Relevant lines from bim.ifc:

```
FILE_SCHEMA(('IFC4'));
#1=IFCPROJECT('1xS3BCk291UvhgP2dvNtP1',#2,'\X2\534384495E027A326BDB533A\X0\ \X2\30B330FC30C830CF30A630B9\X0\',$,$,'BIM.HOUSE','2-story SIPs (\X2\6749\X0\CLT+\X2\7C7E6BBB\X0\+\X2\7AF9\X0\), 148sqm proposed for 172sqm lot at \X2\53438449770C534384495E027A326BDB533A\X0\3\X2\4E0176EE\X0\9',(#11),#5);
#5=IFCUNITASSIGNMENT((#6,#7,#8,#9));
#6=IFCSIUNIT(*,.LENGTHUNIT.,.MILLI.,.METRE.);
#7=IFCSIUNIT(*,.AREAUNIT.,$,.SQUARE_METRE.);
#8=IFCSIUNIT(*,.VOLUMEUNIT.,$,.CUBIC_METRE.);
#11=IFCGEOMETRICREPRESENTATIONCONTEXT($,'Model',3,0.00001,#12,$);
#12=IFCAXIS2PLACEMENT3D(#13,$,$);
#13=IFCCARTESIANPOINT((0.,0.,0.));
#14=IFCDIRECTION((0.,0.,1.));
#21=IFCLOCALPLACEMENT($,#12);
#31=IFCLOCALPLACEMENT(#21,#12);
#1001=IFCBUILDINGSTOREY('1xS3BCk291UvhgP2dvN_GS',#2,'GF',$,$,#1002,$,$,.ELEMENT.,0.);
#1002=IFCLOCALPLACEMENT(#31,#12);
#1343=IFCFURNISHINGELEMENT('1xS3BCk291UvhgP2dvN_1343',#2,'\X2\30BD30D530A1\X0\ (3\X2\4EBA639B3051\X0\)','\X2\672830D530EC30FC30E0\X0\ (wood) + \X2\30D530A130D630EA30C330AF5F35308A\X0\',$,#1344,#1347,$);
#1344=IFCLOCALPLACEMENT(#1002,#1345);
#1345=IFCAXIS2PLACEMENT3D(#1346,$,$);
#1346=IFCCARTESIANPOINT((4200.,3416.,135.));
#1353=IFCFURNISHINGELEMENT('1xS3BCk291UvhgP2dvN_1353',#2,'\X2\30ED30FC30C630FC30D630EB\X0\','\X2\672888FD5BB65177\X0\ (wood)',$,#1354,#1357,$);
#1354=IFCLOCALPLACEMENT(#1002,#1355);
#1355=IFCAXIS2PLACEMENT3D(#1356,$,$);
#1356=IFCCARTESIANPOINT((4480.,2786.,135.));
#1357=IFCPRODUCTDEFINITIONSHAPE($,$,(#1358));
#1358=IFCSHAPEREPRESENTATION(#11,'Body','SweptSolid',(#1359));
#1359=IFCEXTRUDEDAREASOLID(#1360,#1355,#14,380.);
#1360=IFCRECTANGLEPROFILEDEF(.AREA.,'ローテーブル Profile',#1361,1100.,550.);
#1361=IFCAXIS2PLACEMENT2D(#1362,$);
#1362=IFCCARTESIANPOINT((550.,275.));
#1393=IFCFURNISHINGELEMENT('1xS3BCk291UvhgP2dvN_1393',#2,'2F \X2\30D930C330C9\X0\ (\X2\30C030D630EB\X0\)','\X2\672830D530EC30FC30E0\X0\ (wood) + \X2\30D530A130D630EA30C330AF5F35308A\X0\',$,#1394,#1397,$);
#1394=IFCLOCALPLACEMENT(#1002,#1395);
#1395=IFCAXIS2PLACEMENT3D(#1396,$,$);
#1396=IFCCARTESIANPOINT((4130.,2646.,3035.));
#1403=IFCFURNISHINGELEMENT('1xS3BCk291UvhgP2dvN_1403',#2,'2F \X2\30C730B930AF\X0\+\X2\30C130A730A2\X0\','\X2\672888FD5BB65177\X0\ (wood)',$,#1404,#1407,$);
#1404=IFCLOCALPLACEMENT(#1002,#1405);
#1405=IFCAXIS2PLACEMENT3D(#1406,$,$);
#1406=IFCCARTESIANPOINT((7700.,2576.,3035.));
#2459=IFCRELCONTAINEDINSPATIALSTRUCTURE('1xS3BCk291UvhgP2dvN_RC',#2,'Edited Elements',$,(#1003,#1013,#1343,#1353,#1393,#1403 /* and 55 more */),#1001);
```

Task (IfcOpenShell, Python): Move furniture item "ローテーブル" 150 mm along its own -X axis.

```python
import ifcopenshell
import ifcopenshell.api.geometry
import ifcopenshell.util.placement

model = ifcopenshell.open("bim.ifc")

item = model.by_guid("1xS3BCk291UvhgP2dvN_1353")
matrix = ifcopenshell.util.placement.get_local_placement(item.ObjectPlacement)
matrix[:3, 3] -= matrix[:3, 0] * 150.0
ifcopenshell.api.geometry.edit_object_placement(model, product=item, matrix=matrix, is_si=False)

print(ifcopenshell.util.placement.get_local_placement(item.ObjectPlacement).round(3) + 0.0)

model.write("bim_edited.ifc")
```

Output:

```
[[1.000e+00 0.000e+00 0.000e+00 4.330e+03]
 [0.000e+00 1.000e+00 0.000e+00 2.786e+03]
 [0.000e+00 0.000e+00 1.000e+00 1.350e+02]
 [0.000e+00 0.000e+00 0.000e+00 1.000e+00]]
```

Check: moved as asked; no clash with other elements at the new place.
